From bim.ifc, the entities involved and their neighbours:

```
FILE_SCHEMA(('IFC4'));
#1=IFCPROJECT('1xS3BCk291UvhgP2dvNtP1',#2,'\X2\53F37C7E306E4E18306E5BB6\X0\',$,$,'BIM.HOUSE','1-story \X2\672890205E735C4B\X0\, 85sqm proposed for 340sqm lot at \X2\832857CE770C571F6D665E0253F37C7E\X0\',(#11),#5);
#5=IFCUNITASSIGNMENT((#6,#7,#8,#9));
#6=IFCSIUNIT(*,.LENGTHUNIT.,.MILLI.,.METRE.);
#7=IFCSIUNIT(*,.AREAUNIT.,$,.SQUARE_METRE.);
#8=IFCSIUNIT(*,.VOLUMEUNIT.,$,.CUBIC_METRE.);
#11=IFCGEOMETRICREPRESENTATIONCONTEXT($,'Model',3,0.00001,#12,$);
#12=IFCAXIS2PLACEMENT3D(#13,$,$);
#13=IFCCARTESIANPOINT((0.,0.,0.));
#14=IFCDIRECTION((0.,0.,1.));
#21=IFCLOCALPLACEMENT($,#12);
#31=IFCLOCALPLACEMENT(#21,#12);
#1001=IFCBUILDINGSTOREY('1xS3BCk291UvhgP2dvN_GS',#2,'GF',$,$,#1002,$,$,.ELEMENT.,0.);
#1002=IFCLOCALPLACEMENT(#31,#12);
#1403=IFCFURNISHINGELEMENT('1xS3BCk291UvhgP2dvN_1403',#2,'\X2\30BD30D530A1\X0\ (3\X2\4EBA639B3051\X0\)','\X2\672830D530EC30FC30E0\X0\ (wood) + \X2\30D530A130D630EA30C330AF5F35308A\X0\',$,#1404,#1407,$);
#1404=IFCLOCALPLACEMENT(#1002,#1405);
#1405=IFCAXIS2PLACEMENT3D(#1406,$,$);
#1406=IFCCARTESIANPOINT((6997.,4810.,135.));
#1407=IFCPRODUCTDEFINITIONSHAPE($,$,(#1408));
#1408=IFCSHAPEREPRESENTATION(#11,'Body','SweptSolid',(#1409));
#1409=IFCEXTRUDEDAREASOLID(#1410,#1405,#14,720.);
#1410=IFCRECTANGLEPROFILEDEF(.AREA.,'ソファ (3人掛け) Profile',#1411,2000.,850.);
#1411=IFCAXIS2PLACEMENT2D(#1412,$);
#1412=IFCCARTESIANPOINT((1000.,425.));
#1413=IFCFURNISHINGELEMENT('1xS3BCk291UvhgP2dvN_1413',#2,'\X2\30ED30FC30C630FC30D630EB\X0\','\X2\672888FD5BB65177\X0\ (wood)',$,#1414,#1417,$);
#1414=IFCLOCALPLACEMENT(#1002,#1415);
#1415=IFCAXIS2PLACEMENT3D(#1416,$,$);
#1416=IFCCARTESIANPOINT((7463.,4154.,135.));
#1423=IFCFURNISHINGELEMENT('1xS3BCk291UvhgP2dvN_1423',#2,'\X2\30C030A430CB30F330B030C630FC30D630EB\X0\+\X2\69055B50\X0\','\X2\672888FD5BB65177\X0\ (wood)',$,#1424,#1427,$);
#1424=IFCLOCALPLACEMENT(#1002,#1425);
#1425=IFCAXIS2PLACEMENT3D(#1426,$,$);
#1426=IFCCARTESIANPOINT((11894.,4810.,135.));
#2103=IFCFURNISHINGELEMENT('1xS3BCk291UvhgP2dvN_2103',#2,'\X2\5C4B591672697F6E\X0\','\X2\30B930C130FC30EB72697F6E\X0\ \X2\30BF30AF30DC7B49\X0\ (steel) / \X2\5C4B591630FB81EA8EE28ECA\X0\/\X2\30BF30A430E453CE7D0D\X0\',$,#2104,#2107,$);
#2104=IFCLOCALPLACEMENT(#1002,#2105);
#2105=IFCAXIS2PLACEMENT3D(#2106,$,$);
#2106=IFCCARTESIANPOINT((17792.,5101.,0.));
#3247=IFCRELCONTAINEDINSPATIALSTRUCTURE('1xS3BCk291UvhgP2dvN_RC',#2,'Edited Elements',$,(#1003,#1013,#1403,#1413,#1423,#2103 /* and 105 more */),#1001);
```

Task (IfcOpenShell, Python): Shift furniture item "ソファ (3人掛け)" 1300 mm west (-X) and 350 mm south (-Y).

```python
import ifcopenshell
import ifcopenshell.api.geometry
import ifcopenshell.util.placement
import ifcopenshell.util.unit

model = ifcopenshell.open("bim.ifc")
unit_scale = ifcopenshell.util.unit.calculate_unit_scale(model)

item = model.by_guid("1xS3BCk291UvhgP2dvN_1403")
matrix = ifcopenshell.util.placement.get_local_placement(item.ObjectPlacement)
matrix[0, 3] -= 1.3 / unit_scale
matrix[1, 3] -= 0.35 / unit_scale
ifcopenshell.api.geometry.edit_object_placement(model, product=item, matrix=matrix, is_si=False)

print(ifcopenshell.util.placement.get_local_placement(item.ObjectPlacement).round(3) + 0.0)

model.write("bim_updated.ifc")
```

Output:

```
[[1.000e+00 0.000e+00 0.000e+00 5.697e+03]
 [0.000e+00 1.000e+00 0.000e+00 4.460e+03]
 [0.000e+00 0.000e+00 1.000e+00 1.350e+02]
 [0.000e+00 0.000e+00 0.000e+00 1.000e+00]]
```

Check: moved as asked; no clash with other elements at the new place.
